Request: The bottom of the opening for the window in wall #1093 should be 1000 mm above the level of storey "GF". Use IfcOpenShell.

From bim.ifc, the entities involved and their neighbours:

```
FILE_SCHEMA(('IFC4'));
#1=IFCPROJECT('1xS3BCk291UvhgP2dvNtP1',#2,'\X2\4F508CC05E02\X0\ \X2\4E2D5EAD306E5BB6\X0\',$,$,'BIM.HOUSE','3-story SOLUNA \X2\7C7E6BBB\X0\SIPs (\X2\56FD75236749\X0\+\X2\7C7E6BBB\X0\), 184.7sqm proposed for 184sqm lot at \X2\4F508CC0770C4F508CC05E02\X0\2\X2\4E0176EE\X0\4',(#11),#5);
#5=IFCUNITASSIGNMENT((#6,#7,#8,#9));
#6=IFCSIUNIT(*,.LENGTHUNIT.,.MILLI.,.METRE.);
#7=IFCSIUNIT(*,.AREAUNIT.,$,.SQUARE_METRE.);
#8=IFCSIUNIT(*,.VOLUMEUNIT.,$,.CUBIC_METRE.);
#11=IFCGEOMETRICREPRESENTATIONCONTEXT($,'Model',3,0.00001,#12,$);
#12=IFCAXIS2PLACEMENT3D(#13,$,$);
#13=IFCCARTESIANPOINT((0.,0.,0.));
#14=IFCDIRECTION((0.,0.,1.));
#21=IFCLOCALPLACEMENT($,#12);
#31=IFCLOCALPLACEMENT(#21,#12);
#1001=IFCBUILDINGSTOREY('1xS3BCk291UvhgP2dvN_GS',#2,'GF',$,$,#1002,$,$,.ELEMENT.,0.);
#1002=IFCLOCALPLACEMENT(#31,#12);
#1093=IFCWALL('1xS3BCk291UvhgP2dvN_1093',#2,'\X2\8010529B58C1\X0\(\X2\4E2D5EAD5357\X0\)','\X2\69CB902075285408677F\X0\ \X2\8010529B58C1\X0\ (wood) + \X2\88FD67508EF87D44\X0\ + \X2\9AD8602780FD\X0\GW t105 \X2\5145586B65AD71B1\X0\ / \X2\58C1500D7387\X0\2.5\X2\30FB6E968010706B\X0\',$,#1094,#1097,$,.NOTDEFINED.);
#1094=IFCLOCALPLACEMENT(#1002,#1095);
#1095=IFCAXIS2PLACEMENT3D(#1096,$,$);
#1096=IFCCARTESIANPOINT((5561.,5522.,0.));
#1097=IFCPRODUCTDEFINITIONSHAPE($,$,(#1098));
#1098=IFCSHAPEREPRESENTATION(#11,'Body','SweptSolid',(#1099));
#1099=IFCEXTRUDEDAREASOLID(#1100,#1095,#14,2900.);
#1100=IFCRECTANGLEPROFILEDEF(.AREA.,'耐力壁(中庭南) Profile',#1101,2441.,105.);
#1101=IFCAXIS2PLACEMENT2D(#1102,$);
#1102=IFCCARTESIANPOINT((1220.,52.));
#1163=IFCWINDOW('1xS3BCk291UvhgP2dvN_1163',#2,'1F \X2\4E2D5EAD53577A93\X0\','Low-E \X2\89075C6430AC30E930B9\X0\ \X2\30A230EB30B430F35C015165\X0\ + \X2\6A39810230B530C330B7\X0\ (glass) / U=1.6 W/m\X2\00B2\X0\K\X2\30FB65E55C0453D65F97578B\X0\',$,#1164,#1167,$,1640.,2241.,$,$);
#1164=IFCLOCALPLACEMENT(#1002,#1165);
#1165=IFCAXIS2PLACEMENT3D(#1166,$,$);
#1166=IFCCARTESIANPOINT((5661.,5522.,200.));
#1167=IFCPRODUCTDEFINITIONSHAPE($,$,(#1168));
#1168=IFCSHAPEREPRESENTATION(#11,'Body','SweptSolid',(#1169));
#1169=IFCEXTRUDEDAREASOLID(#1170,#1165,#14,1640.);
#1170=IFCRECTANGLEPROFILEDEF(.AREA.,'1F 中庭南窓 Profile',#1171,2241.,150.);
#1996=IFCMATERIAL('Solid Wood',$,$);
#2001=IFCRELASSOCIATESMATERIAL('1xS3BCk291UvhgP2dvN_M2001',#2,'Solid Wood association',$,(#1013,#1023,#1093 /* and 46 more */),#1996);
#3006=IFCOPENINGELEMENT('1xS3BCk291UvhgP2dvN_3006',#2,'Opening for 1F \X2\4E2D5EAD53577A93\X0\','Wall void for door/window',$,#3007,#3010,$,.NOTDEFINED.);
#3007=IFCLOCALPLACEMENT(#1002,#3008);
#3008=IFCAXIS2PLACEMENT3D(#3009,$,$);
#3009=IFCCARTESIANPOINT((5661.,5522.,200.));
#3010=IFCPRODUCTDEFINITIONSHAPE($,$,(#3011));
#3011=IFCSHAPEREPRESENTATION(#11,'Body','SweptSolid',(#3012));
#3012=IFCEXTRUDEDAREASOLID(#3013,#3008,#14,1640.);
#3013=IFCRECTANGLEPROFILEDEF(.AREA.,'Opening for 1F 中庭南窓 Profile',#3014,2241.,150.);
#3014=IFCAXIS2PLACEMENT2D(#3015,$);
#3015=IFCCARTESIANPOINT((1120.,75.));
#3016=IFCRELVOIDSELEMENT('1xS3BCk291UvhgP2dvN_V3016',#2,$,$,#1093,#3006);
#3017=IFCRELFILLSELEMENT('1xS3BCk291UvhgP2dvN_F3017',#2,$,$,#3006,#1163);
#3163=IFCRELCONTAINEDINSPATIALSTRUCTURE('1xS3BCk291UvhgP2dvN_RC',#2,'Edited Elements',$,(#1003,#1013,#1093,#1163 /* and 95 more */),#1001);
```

```python
import numpy as np
import ifcopenshell
import ifcopenshell.api.geometry
import ifcopenshell.geom
import ifcopenshell.util.element
import ifcopenshell.util.placement
import ifcopenshell.util.shape
import ifcopenshell.util.unit

model = ifcopenshell.open("bim.ifc")
unit_scale = ifcopenshell.util.unit.calculate_unit_scale(model)

window = model.by_guid("1xS3BCk291UvhgP2dvN_1163")
opening = window.FillsVoids[0].RelatingOpeningElement
storey = ifcopenshell.util.element.get_container(window, ifc_class="IfcBuildingStorey")
level = ifcopenshell.util.placement.get_local_placement(storey.ObjectPlacement)[2, 3]

# The opening's origin need not be at the sill, so measure its lowest point.
shape = ifcopenshell.geom.create_shape(ifcopenshell.geom.settings(), opening)
bottom = ifcopenshell.util.shape.get_shape_bottom_elevation(shape, shape.geometry) / unit_scale
dz = level + 1 / unit_scale - bottom

shift = np.array([0.0, 0.0, dz])
# The window is not placed relative to its opening, so move both.
for product in (opening, window):
    matrix = ifcopenshell.util.placement.get_local_placement(product.ObjectPlacement)
    matrix[:3, 3] += shift
    ifcopenshell.api.geometry.edit_object_placement(model, product=product, matrix=matrix, is_si=False)

print(f"moved by {dz * unit_scale:+.3f} m")

model.write("bim_v2.ifc")
```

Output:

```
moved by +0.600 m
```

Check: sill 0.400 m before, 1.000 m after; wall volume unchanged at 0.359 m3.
